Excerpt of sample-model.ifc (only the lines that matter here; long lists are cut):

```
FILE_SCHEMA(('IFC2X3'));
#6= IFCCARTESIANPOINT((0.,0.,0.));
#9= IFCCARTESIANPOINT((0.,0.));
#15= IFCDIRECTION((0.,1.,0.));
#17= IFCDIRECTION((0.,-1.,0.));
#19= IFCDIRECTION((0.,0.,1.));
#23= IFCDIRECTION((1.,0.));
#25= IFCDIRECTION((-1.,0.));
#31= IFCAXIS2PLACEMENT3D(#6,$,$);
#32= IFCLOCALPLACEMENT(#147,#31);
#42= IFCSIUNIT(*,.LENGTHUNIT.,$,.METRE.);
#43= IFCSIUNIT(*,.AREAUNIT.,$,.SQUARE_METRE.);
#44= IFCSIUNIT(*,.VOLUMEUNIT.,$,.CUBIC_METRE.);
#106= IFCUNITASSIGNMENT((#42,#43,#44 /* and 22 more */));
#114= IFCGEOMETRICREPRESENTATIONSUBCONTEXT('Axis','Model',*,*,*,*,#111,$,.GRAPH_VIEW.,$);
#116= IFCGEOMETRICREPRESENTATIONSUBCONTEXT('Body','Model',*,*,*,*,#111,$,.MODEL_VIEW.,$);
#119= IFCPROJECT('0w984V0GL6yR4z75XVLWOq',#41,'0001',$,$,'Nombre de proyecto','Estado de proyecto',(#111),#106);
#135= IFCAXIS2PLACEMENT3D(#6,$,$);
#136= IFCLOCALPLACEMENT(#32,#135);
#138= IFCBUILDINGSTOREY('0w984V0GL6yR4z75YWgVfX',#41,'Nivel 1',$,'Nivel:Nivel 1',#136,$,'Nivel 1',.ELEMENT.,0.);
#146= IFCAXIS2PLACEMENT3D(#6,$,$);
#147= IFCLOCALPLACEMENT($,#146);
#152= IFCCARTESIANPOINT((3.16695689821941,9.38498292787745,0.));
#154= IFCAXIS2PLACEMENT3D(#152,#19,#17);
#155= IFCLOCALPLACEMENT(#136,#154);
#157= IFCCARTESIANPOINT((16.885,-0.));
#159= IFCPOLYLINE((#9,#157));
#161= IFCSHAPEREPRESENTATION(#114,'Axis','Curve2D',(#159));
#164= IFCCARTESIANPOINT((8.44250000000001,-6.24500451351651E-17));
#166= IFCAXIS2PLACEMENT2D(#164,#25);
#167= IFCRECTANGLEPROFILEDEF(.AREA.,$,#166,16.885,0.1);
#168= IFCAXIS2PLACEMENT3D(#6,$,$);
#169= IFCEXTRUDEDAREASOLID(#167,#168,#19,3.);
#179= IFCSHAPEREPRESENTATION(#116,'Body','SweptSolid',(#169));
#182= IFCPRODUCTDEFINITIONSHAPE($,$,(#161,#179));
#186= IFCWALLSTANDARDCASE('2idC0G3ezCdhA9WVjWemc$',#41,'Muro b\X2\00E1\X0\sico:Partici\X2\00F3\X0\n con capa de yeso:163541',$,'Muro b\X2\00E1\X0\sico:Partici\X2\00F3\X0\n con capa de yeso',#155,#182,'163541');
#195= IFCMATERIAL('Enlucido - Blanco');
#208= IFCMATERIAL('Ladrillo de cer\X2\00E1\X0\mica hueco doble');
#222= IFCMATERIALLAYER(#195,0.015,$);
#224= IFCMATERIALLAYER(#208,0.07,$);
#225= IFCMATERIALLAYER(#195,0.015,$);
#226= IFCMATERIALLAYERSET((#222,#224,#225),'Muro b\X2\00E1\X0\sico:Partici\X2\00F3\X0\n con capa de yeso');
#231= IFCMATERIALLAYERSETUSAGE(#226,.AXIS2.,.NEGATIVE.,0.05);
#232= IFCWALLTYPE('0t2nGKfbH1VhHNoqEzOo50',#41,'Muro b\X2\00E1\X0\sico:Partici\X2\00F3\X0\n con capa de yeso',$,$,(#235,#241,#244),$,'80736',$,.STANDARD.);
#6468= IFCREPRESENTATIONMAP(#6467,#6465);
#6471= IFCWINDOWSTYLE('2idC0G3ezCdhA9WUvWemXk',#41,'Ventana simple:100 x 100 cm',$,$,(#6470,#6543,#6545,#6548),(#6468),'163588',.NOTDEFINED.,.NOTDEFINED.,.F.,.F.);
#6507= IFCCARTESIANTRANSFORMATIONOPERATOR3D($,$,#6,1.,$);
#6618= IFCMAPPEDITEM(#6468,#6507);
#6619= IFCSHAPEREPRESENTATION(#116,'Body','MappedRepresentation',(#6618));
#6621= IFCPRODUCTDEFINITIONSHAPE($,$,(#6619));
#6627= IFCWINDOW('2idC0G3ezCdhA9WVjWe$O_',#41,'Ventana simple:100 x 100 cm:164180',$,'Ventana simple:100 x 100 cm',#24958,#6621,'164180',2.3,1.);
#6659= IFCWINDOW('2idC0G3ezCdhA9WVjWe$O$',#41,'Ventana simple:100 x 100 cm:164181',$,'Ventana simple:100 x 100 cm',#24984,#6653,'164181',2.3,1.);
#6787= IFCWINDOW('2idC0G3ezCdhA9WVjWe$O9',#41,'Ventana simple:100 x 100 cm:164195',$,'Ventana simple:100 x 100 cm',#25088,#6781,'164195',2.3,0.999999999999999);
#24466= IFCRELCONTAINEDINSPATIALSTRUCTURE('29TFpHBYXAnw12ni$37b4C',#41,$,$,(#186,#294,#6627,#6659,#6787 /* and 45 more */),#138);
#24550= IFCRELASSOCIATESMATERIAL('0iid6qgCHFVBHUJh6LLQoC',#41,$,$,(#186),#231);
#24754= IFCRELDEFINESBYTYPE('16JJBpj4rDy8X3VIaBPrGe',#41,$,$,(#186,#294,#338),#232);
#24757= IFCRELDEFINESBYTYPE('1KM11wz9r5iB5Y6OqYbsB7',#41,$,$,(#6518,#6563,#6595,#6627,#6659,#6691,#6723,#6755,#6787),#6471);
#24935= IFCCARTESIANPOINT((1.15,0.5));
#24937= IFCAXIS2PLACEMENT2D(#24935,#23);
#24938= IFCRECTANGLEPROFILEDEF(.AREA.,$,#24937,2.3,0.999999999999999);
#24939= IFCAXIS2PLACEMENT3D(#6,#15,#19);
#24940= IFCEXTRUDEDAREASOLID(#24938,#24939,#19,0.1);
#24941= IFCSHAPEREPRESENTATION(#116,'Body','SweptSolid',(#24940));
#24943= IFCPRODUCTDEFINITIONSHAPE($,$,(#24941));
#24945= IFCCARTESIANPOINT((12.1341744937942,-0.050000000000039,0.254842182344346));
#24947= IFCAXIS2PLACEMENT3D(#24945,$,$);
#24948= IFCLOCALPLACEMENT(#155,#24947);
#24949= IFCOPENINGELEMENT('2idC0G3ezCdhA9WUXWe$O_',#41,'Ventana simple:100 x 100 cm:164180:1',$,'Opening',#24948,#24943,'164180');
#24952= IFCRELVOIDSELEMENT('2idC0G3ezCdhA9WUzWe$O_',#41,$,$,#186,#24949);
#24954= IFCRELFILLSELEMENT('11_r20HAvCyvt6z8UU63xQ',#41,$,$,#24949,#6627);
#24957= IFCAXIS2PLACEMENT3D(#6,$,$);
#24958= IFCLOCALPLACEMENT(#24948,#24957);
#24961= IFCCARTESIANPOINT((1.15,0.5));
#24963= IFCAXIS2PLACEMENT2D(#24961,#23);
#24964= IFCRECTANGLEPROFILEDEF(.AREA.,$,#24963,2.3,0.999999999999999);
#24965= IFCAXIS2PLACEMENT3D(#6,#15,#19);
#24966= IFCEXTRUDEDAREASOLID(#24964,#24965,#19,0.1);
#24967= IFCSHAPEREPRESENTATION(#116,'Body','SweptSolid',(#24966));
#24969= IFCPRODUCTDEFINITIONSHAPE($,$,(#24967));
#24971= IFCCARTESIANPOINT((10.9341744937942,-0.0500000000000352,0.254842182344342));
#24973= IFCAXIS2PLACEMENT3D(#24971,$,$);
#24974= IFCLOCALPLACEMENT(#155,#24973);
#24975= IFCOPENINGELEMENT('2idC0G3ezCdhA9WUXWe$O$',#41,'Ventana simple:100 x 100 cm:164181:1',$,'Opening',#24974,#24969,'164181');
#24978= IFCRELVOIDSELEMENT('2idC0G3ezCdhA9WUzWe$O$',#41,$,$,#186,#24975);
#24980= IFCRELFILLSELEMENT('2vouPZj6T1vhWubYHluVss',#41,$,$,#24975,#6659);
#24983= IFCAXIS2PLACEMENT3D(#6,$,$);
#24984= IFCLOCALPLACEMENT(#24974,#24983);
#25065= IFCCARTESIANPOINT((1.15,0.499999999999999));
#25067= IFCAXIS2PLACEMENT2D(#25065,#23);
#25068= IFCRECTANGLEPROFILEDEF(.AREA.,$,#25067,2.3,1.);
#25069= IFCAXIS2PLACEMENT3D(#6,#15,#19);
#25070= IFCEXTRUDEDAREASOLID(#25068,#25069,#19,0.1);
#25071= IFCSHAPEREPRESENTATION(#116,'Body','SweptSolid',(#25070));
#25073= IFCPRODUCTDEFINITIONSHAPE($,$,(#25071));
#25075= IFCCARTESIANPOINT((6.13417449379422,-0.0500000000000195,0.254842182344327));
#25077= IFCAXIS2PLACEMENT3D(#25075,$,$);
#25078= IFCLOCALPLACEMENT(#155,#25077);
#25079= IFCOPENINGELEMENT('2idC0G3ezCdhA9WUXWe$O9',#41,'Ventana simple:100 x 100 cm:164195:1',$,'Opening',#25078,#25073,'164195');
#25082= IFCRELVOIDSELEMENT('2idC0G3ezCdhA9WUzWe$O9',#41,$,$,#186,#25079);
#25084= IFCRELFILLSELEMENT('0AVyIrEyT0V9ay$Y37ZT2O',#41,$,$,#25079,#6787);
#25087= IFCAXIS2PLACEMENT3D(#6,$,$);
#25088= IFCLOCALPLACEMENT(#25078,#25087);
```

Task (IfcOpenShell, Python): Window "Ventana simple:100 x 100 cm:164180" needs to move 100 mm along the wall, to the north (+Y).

```python
import ifcopenshell
import ifcopenshell.api.geometry
import ifcopenshell.util.placement
import ifcopenshell.util.unit

model = ifcopenshell.open("sample-model.ifc")
unit_scale = ifcopenshell.util.unit.calculate_unit_scale(model)

window = model.by_id(6627)
opening = window.FillsVoids[0].RelatingOpeningElement
wall = opening.VoidsElements[0].RelatingBuildingElement

wall_matrix = ifcopenshell.util.placement.get_local_placement(wall.ObjectPlacement)
shift = wall_matrix[:3, 0] * -0.1 / unit_scale
before = ifcopenshell.util.placement.get_local_placement(window.ObjectPlacement)[:3, 3].copy()

# The window is placed relative to its opening, so it follows when the opening moves.
matrix = ifcopenshell.util.placement.get_local_placement(opening.ObjectPlacement)
matrix[:3, 3] += shift
ifcopenshell.api.geometry.edit_object_placement(
    model, product=opening, matrix=matrix, is_si=False, should_transform_children=True
)

after = ifcopenshell.util.placement.get_local_placement(window.ObjectPlacement)[:3, 3]
print("window moved by", (after - before).round(3) + 0.0)

model.write("sample-model_updated.ifc")
```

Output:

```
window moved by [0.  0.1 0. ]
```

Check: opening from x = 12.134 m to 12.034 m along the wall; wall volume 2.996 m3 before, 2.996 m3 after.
